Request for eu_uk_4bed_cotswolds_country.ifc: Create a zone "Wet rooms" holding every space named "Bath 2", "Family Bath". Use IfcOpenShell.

First a look at what the model holds.

```python
import ifcopenshell

model = ifcopenshell.open("eu_uk_4bed_cotswolds_country.ifc")
print(model.schema)
seen = {}
for space in model.by_type("IfcSpace"):
    seen[space.LongName] = seen.get(space.LongName, 0) + 1
for name, count in sorted(seen.items(), key=str):
    print(count, "x", name)
print("zones:", [z.Name for z in model.by_type("IfcZone")][:20])
```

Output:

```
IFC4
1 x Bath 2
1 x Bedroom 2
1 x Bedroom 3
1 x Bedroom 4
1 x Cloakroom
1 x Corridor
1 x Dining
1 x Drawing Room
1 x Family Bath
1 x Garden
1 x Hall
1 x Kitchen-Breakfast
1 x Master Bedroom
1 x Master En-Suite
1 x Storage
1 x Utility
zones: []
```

```python
import ifcopenshell
import ifcopenshell.api.group
import ifcopenshell.api.root

model = ifcopenshell.open("eu_uk_4bed_cotswolds_country.ifc")

names = {"Bath 2", "Family Bath"}
spaces = [s for s in model.by_type("IfcSpace") if s.LongName in names]

zone = ifcopenshell.api.root.create_entity(model, ifc_class="IfcZone", name="Wet rooms")
ifcopenshell.api.group.assign_group(model, products=spaces, group=zone)
print(len(spaces), "spaces in", zone.Name)

model.write("eu_uk_4bed_cotswolds_country_edited.ifc")
```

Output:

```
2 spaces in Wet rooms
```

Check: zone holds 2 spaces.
